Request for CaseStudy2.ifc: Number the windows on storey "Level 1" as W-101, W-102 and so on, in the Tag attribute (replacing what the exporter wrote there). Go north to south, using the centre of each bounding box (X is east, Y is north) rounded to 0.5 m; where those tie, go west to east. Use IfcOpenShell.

First a look at what the model holds.

```python
import ifcopenshell
import ifcopenshell.util.element
import ifcopenshell.util.placement

model = ifcopenshell.open("CaseStudy2.ifc")
print(model.schema)
storey = next(s for s in model.by_type("IfcBuildingStorey") if s.Name == "Level 1")
windows = [e for e in ifcopenshell.util.element.get_decomposition(storey) if e.is_a("IfcWindow")]
for e in sorted(windows, key=lambda e: e.id()):
    origin = ifcopenshell.util.placement.get_local_placement(e.ObjectPlacement)[:3, 3]
    print(e.id(), e.Tag, e.Name, origin.round(2) + 0.0, sep=" | ")
```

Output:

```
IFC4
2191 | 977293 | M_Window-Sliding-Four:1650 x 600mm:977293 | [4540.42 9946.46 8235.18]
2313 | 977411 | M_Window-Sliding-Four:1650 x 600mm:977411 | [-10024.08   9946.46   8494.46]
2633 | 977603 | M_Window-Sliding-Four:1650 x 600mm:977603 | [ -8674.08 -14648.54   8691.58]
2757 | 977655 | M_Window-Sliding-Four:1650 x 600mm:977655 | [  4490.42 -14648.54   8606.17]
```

```python
import ifcopenshell
import ifcopenshell.geom
import ifcopenshell.util.element
import ifcopenshell.util.shape

model = ifcopenshell.open("CaseStudy2.ifc")
settings = ifcopenshell.geom.settings()
settings.set("use-world-coords", True)


def centre(element):
    shape = ifcopenshell.geom.create_shape(settings, element)
    return ifcopenshell.util.shape.get_bbox_centroid(shape.geometry)


storey = next(s for s in model.by_type("IfcBuildingStorey") if s.Name == "Level 1")
windows = [e for e in ifcopenshell.util.element.get_decomposition(storey) if e.is_a("IfcWindow")]

# Insertion points can sit at a corner or the storey origin, so sort by the geometry (in metres).
centres = {e: centre(e) for e in windows}
windows.sort(key=lambda e: (-round(centres[e][1] / 0.5), centres[e][0]))

for i, e in enumerate(windows, start=1):
    number = f"W-1{i:02d}"
    e.Tag = number
    print(e.id(), number)

model.write("CaseStudy2_updated.ifc")
```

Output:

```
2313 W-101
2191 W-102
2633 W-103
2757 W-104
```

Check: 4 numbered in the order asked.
